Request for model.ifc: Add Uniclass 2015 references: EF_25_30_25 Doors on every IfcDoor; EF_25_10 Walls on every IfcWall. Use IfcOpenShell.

First a look at what the model holds.

```python
import ifcopenshell

model = ifcopenshell.open("model.ifc")
print(model.schema)
print("classifications:", [c.Name for c in model.by_type("IfcClassification")])
for ifc_class in ("IfcDoor", "IfcRoof", "IfcStair", "IfcWall", "IfcWindow"):
    print(ifc_class, len(model.by_type(ifc_class)))
```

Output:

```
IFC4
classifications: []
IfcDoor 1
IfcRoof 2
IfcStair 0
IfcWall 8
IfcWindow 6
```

```python
import ifcopenshell
import ifcopenshell.api.classification

model = ifcopenshell.open("model.ifc")

system = ifcopenshell.api.classification.add_classification(model, classification="Uniclass 2015")

codes = {
    "IfcDoor": ("EF_25_30_25", "Doors"),
    "IfcWall": ("EF_25_10", "Walls"),
}
for ifc_class, (code, name) in codes.items():
    products = model.by_type(ifc_class)
    ifcopenshell.api.classification.add_reference(
        model, products=products, classification=system, identification=code, name=name
    )
    print(code, len(products))

model.write("model_edited.ifc")
```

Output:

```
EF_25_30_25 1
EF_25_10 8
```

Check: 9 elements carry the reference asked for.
